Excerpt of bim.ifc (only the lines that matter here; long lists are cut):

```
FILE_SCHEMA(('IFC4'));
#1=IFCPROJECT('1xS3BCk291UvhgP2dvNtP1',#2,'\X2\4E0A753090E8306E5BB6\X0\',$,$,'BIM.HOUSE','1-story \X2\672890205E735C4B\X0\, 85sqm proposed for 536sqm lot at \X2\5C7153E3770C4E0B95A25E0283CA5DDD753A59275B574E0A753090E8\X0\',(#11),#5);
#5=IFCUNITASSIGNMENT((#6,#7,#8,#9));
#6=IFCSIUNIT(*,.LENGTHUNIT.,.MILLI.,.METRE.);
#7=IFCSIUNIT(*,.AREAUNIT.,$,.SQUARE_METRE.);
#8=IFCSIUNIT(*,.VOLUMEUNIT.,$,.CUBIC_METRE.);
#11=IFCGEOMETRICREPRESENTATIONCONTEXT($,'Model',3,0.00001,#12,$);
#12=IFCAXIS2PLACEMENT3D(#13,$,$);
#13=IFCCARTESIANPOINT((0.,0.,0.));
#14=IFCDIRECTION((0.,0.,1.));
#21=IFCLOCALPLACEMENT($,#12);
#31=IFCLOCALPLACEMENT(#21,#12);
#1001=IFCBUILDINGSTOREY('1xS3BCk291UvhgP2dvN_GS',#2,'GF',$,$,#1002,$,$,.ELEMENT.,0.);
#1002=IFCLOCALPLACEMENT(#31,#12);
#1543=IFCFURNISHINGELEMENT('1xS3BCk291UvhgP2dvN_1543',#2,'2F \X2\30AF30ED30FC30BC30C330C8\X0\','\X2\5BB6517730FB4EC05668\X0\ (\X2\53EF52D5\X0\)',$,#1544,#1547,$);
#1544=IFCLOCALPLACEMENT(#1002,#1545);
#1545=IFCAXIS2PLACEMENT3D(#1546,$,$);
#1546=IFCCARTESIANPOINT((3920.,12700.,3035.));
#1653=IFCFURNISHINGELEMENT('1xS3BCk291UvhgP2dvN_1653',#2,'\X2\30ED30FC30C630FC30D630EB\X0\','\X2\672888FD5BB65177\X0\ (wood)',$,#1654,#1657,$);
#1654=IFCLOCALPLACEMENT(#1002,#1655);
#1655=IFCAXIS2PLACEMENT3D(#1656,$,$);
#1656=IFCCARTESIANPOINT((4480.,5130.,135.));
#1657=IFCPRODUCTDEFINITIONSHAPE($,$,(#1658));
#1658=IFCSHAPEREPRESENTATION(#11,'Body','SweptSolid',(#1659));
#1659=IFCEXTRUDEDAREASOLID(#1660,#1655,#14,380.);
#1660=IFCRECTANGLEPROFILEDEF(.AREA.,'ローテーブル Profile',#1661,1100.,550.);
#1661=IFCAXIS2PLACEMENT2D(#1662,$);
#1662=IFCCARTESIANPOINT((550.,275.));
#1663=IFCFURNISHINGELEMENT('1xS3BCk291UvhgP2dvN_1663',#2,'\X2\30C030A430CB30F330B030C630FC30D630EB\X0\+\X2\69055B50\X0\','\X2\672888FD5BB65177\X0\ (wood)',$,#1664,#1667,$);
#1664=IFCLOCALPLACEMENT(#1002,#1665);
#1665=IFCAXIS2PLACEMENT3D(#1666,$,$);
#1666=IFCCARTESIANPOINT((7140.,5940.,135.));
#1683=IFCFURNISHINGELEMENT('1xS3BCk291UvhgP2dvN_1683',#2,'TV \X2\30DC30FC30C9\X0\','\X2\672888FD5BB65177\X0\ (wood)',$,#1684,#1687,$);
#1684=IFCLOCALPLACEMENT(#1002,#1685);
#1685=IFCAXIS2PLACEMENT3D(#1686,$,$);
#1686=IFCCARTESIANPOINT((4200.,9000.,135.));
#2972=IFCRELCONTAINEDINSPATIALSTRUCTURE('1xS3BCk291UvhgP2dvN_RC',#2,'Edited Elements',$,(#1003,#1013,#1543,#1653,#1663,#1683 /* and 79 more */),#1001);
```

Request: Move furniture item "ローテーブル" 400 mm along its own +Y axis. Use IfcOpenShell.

```python
import ifcopenshell
import ifcopenshell.api.geometry
import ifcopenshell.util.placement
import ifcopenshell.util.unit

model = ifcopenshell.open("bim.ifc")
unit_scale = ifcopenshell.util.unit.calculate_unit_scale(model)

item = model.by_guid("1xS3BCk291UvhgP2dvN_1653")
matrix = ifcopenshell.util.placement.get_local_placement(item.ObjectPlacement)
matrix[:3, 3] += matrix[:3, 1] * 0.4 / unit_scale
ifcopenshell.api.geometry.edit_object_placement(model, product=item, matrix=matrix, is_si=False)

print(ifcopenshell.util.placement.get_local_placement(item.ObjectPlacement).round(3) + 0.0)

model.write("bim-out.ifc")
```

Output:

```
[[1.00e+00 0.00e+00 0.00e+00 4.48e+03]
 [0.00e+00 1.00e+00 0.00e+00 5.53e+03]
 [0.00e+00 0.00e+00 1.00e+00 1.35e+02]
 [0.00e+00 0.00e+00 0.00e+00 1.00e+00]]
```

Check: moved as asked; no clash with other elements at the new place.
